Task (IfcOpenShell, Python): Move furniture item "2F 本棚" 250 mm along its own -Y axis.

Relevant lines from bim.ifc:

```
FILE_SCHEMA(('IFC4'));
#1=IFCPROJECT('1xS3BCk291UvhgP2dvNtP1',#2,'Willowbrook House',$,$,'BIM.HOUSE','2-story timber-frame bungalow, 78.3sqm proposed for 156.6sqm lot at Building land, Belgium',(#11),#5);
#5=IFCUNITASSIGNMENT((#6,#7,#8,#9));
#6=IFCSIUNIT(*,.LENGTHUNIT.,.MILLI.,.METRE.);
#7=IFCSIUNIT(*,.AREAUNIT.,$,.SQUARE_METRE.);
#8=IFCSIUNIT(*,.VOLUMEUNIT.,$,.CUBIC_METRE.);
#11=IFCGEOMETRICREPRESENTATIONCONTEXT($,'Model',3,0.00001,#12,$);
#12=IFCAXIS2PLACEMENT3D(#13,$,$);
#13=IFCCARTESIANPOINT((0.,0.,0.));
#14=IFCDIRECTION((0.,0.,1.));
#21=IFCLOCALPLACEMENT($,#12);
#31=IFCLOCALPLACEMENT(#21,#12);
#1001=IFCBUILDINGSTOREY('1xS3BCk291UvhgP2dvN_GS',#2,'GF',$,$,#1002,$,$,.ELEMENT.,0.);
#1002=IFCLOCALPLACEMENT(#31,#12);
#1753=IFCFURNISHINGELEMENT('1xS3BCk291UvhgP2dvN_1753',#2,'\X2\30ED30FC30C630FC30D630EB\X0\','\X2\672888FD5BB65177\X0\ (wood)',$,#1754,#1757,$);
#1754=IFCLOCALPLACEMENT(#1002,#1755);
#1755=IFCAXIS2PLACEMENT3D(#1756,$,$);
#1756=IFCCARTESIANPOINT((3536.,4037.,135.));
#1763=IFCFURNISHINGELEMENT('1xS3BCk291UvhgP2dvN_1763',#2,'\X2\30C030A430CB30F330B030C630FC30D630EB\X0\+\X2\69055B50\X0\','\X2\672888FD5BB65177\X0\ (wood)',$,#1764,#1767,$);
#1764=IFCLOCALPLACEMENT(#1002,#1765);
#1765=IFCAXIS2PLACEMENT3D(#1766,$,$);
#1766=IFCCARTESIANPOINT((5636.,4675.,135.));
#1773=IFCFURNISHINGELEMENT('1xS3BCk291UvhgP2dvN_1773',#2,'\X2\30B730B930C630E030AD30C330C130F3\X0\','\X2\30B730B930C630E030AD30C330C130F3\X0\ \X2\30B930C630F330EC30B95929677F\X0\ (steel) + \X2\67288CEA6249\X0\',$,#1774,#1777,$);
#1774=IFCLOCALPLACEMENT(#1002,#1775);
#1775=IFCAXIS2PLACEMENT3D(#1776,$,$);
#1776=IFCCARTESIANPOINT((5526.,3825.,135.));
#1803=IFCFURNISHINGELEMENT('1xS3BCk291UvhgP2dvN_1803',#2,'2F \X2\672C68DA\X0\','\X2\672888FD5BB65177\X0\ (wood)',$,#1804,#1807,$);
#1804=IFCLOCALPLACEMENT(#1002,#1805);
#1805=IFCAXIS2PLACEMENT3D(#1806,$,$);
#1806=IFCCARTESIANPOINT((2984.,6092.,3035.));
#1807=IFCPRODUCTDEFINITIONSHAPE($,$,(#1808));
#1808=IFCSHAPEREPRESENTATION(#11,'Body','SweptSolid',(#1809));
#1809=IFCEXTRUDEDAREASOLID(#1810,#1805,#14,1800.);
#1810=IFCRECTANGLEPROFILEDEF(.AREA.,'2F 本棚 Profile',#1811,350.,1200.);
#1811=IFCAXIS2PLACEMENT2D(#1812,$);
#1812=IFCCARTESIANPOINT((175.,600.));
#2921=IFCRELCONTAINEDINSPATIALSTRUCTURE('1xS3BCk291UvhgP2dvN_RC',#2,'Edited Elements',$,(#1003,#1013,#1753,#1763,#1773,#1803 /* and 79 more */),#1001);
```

```python
import ifcopenshell
import ifcopenshell.api.geometry
import ifcopenshell.util.placement
import ifcopenshell.util.unit

model = ifcopenshell.open("bim.ifc")
unit_scale = ifcopenshell.util.unit.calculate_unit_scale(model)

item = model.by_id(1803)
matrix = ifcopenshell.util.placement.get_local_placement(item.ObjectPlacement)
matrix[:3, 3] -= matrix[:3, 1] * 0.25 / unit_scale
ifcopenshell.api.geometry.edit_object_placement(model, product=item, matrix=matrix, is_si=False)

print(ifcopenshell.util.placement.get_local_placement(item.ObjectPlacement).round(3) + 0.0)

model.write("bim_rev.ifc")
```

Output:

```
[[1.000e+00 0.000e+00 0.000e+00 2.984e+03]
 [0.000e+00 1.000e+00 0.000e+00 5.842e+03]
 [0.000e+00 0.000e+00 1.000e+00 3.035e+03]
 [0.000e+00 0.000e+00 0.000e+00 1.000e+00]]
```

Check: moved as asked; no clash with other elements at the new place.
